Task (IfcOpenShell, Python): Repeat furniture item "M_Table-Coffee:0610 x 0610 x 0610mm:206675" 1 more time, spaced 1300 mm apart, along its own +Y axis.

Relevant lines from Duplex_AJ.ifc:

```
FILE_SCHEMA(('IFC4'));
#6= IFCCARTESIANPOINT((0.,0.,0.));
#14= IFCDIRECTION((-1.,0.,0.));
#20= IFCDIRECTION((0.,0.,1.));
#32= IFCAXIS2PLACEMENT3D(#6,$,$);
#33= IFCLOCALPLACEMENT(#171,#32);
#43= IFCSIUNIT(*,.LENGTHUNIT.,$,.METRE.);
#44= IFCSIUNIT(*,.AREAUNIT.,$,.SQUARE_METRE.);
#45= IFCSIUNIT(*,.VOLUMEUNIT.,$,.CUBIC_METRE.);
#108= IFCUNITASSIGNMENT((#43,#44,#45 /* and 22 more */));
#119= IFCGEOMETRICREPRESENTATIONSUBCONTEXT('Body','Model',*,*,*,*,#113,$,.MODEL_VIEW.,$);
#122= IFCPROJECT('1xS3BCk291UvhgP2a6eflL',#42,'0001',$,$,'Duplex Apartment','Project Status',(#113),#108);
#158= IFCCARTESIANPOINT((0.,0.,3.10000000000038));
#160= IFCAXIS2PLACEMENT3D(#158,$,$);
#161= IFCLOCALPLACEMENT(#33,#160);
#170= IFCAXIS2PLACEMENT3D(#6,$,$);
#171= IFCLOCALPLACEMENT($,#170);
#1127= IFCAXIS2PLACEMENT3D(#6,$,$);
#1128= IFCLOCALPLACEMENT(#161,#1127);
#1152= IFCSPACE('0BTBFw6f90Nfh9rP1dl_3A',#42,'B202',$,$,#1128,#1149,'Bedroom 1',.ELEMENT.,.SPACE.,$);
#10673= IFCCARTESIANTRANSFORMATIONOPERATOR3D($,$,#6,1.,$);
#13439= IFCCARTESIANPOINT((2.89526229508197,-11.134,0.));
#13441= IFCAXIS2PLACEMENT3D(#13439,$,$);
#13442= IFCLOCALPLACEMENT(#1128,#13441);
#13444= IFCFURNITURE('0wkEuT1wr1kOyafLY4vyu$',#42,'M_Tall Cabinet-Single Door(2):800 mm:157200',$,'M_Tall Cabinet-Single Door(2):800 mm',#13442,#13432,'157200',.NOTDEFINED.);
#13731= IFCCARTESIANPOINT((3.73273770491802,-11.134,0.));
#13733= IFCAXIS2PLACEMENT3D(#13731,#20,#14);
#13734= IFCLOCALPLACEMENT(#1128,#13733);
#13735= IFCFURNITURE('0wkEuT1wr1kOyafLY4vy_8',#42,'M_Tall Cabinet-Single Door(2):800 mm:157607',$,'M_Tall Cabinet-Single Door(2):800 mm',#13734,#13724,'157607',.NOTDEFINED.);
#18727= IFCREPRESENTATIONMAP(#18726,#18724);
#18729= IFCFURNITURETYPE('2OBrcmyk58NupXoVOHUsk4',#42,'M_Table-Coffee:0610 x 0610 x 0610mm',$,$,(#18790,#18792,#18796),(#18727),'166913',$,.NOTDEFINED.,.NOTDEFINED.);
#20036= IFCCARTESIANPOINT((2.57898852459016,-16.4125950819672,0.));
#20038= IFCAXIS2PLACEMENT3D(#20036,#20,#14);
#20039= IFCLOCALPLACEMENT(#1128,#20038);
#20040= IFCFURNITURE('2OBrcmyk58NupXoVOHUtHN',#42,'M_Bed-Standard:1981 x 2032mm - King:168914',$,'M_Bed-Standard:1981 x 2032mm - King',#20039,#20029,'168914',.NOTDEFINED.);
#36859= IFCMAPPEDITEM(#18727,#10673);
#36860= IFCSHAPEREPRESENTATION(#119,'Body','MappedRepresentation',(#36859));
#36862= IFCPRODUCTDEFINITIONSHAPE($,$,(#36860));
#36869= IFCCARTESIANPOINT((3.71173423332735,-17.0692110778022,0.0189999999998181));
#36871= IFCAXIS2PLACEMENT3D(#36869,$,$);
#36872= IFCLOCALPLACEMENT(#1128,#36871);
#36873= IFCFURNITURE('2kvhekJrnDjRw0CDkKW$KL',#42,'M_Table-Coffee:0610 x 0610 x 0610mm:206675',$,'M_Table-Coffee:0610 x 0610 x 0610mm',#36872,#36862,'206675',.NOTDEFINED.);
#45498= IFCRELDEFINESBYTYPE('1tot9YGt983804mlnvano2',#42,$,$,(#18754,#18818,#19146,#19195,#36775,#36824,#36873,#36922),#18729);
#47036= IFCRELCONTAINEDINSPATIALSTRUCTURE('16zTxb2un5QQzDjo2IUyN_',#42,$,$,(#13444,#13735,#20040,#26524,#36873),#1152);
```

```python
import ifcopenshell
import ifcopenshell.api.geometry
import ifcopenshell.api.root
import ifcopenshell.util.element
import ifcopenshell.util.placement
import ifcopenshell.util.unit

model = ifcopenshell.open("Duplex_AJ.ifc")
unit_scale = ifcopenshell.util.unit.calculate_unit_scale(model)


def reuse_history(source, copy):
    """copy_class also copies each property set's owner history, people and application; keep the originals."""
    for rel in copy.IsDefinedBy:
        if rel.is_a("IfcRelDefinesByProperties") and (history := rel.RelatingPropertyDefinition.OwnerHistory):
            rel.RelatingPropertyDefinition.OwnerHistory = source.OwnerHistory
            ifcopenshell.util.element.remove_deep2(model, history)


source = model.by_guid("2kvhekJrnDjRw0CDkKW$KL")
base = ifcopenshell.util.placement.get_local_placement(source.ObjectPlacement)
step = base[:3, 1] * 1.3 / unit_scale

for i in range(1, 2):
    copy = ifcopenshell.api.root.copy_class(model, product=source)
    copy.Representation = ifcopenshell.util.element.copy_deep(
        model, source.Representation, exclude=["IfcGeometricRepresentationContext", "IfcRepresentationMap"]
    )
    copy.Name = "M_Table-Coffee:0610 x 0610 x 0610mm"
    copy.Tag = None
    reuse_history(source, copy)
    matrix = base.copy()
    matrix[:3, 3] += i * step
    print("added at", matrix[:3, 3].round(3) + 0.0)
    ifcopenshell.api.geometry.edit_object_placement(model, product=copy, matrix=matrix, is_si=False)

model.write("Duplex_AJ_rev.ifc")
```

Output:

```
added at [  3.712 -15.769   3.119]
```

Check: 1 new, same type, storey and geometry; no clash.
